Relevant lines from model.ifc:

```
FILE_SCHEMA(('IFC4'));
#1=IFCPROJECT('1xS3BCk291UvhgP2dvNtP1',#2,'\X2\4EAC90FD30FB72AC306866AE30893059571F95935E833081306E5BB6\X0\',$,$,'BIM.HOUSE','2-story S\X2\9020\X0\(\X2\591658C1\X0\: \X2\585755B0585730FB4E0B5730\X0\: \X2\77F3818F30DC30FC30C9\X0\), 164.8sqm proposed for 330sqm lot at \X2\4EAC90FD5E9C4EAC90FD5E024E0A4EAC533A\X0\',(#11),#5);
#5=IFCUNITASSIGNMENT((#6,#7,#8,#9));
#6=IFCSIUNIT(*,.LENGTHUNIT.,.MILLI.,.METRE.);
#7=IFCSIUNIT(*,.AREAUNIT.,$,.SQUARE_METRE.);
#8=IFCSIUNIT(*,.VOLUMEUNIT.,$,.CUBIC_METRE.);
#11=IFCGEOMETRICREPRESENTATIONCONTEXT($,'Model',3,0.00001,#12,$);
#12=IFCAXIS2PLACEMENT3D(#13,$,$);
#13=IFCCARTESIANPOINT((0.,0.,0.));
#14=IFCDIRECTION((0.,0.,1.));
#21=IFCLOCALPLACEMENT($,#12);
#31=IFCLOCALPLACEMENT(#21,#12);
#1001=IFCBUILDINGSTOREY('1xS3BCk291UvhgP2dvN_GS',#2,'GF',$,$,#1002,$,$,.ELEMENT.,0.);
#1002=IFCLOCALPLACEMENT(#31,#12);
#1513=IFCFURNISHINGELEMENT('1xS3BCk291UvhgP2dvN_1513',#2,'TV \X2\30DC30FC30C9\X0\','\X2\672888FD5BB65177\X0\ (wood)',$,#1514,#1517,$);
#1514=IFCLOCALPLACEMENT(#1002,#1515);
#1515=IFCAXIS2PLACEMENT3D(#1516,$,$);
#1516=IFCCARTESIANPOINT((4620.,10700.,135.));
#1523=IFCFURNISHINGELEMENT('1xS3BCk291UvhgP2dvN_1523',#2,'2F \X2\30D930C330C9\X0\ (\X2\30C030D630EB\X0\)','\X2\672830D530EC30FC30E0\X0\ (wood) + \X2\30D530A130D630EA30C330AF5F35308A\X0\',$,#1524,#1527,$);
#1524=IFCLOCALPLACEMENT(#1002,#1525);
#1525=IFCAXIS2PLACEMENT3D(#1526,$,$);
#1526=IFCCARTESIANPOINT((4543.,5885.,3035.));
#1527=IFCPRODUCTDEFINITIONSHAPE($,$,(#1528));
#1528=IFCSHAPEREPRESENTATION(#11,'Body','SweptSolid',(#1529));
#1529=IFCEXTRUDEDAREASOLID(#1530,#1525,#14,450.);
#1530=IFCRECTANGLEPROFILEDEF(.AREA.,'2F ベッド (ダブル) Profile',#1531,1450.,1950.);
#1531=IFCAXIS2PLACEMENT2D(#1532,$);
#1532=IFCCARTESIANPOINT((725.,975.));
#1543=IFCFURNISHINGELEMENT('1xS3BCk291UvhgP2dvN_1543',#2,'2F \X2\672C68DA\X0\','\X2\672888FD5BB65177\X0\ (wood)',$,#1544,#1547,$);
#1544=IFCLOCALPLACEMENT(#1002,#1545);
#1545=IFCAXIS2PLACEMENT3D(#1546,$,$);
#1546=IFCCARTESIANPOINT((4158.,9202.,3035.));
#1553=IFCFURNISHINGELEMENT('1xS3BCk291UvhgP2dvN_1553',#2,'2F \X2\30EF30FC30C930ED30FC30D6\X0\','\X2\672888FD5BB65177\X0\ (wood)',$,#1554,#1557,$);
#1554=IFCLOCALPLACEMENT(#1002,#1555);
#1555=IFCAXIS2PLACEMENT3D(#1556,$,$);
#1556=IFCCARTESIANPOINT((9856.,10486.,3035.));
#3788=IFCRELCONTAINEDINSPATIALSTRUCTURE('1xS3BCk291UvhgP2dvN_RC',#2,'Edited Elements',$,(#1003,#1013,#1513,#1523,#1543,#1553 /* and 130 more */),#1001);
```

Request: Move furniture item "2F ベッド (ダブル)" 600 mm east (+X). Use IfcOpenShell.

```python
import ifcopenshell
import ifcopenshell.api.geometry
import ifcopenshell.util.placement
import ifcopenshell.util.unit

model = ifcopenshell.open("model.ifc")
unit_scale = ifcopenshell.util.unit.calculate_unit_scale(model)

item = model.by_id(1523)
matrix = ifcopenshell.util.placement.get_local_placement(item.ObjectPlacement)
matrix[0, 3] += 0.6 / unit_scale
ifcopenshell.api.geometry.edit_object_placement(model, product=item, matrix=matrix, is_si=False)

print(ifcopenshell.util.placement.get_local_placement(item.ObjectPlacement).round(3) + 0.0)

model.write("model_v2.ifc")
```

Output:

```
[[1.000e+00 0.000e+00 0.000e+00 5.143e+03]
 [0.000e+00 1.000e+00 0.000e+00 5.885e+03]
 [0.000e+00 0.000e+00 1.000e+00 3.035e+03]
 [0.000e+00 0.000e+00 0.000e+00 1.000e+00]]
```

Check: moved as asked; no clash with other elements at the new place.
